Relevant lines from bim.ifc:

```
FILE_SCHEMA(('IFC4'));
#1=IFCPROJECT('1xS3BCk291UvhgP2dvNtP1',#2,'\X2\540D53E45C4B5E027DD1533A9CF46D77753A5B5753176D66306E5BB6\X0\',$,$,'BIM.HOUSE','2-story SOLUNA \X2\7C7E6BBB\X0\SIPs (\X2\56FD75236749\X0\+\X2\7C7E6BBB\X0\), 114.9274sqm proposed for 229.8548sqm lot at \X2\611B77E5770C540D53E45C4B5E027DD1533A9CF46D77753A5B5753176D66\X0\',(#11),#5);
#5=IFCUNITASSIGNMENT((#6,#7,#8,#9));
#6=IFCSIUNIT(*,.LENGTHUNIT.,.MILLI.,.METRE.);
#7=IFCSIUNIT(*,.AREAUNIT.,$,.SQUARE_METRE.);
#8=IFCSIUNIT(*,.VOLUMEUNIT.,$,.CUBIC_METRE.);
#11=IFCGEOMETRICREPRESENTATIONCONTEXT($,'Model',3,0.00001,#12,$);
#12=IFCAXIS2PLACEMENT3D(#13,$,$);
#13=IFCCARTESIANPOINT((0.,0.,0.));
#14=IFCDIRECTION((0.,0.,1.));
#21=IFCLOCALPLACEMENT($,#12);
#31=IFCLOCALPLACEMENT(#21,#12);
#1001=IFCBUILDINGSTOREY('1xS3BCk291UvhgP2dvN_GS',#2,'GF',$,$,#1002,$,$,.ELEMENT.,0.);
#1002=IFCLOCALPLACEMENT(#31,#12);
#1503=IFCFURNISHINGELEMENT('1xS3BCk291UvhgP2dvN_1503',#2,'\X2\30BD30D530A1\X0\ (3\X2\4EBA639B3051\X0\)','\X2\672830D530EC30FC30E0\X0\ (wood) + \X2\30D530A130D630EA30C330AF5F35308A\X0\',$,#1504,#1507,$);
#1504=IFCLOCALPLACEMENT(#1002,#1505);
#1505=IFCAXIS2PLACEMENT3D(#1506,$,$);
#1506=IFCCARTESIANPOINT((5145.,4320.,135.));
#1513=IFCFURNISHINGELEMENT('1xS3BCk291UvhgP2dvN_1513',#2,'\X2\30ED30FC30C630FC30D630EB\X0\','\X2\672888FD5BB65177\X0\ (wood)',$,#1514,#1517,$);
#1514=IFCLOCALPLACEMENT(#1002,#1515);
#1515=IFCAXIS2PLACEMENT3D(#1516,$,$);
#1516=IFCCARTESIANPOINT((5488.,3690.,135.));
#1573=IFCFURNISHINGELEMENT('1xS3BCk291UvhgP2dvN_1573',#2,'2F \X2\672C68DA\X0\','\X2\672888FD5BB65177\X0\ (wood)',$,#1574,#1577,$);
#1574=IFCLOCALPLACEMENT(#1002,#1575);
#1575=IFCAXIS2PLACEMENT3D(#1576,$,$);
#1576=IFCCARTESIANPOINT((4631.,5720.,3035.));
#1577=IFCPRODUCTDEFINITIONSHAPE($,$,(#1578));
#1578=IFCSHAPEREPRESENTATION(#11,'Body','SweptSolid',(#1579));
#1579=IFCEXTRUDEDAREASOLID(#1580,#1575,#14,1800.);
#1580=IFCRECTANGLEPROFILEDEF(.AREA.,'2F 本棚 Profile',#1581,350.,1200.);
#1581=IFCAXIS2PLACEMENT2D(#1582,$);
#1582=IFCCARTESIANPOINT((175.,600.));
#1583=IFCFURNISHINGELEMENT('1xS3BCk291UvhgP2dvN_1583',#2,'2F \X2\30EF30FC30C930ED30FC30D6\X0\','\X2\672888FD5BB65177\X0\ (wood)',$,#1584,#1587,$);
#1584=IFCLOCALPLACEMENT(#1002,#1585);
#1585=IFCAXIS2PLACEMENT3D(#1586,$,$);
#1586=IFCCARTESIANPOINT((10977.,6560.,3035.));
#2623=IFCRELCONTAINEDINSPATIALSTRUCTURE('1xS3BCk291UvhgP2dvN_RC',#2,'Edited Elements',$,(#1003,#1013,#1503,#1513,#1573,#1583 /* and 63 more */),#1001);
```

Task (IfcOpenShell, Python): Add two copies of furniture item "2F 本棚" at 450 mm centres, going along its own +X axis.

```python
import ifcopenshell
import ifcopenshell.api.geometry
import ifcopenshell.api.root
import ifcopenshell.util.element
import ifcopenshell.util.placement

model = ifcopenshell.open("bim.ifc")


def reuse_history(source, copy):
    """copy_class also copies each property set's owner history, people and application; keep the originals."""
    for rel in copy.IsDefinedBy:
        if rel.is_a("IfcRelDefinesByProperties") and (history := rel.RelatingPropertyDefinition.OwnerHistory):
            rel.RelatingPropertyDefinition.OwnerHistory = source.OwnerHistory
            ifcopenshell.util.element.remove_deep2(model, history)


source = model.by_guid("1xS3BCk291UvhgP2dvN_1573")
base = ifcopenshell.util.placement.get_local_placement(source.ObjectPlacement)
step = base[:3, 0] * 450.0

for i in range(1, 3):
    copy = ifcopenshell.api.root.copy_class(model, product=source)
    copy.Representation = ifcopenshell.util.element.copy_deep(
        model, source.Representation, exclude=["IfcGeometricRepresentationContext", "IfcRepresentationMap"]
    )
    reuse_history(source, copy)
    matrix = base.copy()
    matrix[:3, 3] += i * step
    print("added at", matrix[:3, 3].round(3) + 0.0)
    ifcopenshell.api.geometry.edit_object_placement(model, product=copy, matrix=matrix, is_si=False)

model.write("bim-out.ifc")
```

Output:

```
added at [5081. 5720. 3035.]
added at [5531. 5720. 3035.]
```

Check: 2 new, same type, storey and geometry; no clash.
